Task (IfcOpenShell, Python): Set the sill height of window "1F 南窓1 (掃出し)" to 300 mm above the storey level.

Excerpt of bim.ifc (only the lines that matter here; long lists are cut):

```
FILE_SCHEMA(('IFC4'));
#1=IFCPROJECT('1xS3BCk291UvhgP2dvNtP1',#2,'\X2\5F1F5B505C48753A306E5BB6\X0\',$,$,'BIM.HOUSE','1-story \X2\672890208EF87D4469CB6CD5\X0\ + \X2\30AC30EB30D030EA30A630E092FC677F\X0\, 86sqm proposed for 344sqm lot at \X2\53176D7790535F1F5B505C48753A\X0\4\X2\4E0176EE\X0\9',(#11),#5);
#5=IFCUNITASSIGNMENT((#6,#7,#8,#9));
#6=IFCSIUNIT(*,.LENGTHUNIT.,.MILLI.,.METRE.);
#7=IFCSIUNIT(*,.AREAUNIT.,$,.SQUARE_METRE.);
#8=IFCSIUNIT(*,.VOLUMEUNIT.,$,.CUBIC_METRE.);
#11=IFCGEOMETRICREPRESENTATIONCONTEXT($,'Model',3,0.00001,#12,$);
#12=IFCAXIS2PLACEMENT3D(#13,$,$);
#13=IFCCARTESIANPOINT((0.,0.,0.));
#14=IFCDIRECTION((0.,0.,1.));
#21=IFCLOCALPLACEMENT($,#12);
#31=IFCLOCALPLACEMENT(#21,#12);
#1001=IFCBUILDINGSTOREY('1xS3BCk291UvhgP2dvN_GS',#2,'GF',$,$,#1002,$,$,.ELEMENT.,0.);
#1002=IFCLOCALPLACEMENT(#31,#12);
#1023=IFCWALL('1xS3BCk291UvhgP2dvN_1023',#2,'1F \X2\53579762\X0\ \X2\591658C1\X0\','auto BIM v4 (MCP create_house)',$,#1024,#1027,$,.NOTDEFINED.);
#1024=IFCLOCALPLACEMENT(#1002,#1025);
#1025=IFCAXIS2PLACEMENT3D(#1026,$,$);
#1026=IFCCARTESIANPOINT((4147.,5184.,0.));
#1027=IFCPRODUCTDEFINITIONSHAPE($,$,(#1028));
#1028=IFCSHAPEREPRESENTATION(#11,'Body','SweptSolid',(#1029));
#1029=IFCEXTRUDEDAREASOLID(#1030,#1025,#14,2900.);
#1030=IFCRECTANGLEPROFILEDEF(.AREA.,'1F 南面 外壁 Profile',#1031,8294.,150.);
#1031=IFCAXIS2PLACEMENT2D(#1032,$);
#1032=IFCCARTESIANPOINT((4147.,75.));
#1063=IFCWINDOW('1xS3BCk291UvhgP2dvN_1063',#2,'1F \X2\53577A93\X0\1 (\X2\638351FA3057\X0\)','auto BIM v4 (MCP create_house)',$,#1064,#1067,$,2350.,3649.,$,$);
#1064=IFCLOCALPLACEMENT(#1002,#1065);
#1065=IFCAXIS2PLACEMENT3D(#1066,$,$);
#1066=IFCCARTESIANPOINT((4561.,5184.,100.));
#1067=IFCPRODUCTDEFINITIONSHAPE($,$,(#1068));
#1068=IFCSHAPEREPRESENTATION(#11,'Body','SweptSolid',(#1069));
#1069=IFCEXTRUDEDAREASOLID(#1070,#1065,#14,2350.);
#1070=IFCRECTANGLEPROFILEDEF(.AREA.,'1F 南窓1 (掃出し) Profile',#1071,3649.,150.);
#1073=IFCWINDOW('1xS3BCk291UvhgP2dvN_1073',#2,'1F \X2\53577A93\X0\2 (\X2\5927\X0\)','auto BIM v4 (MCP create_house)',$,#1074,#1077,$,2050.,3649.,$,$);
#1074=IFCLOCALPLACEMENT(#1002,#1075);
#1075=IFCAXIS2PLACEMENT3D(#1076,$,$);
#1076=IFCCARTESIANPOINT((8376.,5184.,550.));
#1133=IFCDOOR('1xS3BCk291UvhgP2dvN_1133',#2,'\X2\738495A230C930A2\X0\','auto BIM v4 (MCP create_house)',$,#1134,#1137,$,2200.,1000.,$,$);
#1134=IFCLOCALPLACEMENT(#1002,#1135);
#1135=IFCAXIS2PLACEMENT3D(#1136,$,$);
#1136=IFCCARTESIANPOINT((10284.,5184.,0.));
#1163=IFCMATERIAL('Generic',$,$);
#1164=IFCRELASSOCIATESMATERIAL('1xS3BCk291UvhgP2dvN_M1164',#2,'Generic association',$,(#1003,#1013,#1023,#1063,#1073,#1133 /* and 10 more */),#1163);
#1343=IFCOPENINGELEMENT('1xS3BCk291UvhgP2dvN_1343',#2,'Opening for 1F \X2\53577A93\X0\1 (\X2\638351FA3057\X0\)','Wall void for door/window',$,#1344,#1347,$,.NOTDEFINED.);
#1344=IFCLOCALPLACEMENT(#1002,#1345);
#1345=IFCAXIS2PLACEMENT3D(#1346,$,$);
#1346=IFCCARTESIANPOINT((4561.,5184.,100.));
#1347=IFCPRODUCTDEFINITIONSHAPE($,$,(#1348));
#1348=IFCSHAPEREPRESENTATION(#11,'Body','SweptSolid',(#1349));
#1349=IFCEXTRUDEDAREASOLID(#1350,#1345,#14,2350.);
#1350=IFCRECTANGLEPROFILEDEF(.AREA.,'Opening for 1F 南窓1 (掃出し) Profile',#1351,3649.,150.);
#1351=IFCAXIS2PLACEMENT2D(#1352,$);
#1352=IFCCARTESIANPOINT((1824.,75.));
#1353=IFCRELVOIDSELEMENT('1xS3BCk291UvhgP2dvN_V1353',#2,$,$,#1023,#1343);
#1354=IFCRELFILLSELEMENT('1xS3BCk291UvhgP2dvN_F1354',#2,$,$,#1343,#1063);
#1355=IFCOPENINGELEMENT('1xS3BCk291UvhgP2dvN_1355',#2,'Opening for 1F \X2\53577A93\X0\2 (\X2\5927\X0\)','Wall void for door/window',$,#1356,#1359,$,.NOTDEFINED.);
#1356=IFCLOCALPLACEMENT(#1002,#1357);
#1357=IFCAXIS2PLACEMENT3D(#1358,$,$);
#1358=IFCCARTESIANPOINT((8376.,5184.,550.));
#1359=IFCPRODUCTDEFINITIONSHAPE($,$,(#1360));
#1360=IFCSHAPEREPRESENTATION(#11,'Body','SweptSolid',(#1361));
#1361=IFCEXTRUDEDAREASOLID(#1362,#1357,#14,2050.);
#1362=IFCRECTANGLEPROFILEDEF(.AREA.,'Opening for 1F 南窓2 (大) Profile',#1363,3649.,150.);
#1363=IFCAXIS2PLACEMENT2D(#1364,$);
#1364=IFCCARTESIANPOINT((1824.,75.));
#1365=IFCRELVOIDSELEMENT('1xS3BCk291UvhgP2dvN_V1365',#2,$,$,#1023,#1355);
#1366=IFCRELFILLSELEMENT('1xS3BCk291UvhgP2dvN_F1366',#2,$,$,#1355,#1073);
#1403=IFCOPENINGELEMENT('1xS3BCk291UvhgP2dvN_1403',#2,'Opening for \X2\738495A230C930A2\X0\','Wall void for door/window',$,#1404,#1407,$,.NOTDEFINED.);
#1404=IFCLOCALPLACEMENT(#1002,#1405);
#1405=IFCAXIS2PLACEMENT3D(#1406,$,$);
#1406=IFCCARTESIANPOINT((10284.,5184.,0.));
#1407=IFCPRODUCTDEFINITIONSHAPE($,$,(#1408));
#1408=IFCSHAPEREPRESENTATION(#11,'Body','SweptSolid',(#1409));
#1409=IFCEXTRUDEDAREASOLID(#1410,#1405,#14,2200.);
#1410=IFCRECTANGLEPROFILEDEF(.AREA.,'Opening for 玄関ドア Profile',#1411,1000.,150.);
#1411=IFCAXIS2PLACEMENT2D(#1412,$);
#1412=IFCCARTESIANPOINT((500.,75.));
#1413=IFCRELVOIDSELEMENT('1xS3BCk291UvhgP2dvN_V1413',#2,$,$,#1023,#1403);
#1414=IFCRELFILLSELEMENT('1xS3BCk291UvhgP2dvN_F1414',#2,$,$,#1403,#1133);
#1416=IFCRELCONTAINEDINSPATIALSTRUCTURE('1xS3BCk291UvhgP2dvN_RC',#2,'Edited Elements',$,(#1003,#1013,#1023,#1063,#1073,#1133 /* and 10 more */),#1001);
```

```python
import numpy as np
import ifcopenshell
import ifcopenshell.api.geometry
import ifcopenshell.geom
import ifcopenshell.util.element
import ifcopenshell.util.placement
import ifcopenshell.util.shape
import ifcopenshell.util.unit

model = ifcopenshell.open("bim.ifc")
unit_scale = ifcopenshell.util.unit.calculate_unit_scale(model)

window = model.by_guid("1xS3BCk291UvhgP2dvN_1063")
opening = window.FillsVoids[0].RelatingOpeningElement
storey = ifcopenshell.util.element.get_container(window, ifc_class="IfcBuildingStorey")
level = ifcopenshell.util.placement.get_local_placement(storey.ObjectPlacement)[2, 3]

# The opening's origin need not be at the sill, so measure its lowest point.
shape = ifcopenshell.geom.create_shape(ifcopenshell.geom.settings(), opening)
bottom = ifcopenshell.util.shape.get_shape_bottom_elevation(shape, shape.geometry) / unit_scale
dz = level + 0.3 / unit_scale - bottom

shift = np.array([0.0, 0.0, dz])
# The window is not placed relative to its opening, so move both.
for product in (opening, window):
    matrix = ifcopenshell.util.placement.get_local_placement(product.ObjectPlacement)
    matrix[:3, 3] += shift
    ifcopenshell.api.geometry.edit_object_placement(model, product=product, matrix=matrix, is_si=False)

print(f"moved by {dz * unit_scale:+.3f} m")

model.write("bim_edited.ifc")
```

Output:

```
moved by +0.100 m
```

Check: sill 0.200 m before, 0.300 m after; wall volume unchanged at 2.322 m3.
